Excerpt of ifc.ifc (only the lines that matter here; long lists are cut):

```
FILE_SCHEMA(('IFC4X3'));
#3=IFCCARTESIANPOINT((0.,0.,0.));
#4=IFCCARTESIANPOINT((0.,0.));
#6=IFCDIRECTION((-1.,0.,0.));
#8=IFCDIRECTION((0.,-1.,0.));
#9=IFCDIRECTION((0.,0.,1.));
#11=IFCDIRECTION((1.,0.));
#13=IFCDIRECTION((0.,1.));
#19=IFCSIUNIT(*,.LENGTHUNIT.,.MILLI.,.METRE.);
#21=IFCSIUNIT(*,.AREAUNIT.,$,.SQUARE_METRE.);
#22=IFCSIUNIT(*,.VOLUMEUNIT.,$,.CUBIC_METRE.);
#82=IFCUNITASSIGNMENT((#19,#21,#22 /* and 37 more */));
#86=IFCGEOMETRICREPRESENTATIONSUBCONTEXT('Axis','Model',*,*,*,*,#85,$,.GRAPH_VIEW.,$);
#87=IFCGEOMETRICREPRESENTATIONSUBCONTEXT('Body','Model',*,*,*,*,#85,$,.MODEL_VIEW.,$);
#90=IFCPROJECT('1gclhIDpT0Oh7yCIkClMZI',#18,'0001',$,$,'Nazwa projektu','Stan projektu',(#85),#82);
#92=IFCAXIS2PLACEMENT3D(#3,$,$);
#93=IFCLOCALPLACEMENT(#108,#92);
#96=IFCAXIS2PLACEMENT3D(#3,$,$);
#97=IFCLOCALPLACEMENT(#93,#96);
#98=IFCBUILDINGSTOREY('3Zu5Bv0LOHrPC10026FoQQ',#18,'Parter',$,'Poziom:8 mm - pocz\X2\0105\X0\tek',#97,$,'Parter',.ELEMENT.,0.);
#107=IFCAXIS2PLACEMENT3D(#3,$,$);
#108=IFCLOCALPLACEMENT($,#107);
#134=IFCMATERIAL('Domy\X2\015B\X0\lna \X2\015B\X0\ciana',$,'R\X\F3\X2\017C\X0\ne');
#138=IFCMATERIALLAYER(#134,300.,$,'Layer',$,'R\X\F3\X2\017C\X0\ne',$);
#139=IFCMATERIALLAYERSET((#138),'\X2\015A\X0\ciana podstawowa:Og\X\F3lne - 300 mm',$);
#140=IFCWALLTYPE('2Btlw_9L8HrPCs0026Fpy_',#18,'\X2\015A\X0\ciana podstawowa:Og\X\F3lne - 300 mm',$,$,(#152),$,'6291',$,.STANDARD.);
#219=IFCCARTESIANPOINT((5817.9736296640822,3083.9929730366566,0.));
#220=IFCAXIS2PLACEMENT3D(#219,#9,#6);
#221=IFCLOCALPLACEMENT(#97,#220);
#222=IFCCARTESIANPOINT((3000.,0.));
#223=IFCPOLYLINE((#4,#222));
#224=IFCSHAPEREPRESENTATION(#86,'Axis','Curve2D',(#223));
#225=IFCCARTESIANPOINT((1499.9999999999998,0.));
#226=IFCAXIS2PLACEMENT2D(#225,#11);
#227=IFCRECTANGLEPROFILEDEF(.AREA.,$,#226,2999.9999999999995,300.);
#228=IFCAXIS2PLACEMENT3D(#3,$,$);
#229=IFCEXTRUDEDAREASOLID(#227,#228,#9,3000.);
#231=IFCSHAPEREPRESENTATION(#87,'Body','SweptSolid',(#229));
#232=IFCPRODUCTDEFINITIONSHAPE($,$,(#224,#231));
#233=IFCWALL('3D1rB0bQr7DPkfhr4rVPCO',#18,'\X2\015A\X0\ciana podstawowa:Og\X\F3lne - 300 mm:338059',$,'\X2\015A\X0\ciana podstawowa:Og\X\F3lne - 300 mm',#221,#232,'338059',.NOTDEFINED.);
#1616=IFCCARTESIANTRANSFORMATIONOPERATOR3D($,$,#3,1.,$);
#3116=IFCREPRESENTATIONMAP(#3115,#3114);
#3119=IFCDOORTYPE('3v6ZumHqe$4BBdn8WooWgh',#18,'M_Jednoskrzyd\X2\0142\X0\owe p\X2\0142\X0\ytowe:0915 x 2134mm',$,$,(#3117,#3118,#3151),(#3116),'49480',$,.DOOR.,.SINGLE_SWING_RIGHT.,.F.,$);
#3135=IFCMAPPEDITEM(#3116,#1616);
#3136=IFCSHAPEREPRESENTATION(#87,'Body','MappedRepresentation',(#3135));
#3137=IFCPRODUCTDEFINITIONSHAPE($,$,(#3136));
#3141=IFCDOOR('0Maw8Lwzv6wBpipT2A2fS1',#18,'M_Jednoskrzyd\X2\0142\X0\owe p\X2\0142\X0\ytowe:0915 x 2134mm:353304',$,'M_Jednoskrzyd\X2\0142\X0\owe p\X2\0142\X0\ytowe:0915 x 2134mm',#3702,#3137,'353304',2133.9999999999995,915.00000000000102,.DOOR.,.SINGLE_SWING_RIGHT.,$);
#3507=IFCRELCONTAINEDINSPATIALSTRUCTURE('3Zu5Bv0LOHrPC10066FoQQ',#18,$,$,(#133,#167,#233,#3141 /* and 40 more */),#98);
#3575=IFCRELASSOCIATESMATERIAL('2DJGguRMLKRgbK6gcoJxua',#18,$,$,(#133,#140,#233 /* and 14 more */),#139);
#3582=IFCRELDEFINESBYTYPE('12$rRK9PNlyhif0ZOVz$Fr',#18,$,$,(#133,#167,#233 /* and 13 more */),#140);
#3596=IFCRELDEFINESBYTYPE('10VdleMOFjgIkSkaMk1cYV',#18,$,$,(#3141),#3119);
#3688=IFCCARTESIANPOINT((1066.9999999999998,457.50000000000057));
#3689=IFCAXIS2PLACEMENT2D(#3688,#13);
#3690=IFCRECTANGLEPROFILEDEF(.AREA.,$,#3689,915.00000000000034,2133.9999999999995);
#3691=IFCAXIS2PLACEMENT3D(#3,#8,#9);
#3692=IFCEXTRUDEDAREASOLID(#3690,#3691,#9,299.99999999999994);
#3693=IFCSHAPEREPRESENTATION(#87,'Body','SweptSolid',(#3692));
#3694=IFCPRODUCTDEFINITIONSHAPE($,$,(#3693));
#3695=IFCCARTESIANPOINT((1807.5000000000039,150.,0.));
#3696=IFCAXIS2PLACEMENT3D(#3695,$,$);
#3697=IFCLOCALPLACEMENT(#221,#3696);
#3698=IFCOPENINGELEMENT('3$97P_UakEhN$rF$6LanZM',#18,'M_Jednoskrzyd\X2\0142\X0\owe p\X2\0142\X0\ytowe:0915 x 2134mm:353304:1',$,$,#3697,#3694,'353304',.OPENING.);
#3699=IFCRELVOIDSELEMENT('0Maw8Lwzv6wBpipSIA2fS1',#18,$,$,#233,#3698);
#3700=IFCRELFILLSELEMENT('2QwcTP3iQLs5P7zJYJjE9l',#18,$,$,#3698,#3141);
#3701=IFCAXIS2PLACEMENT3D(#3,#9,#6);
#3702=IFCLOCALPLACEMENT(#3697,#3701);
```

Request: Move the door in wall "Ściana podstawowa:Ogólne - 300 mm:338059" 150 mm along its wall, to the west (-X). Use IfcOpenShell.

```python
import ifcopenshell
import ifcopenshell.api.geometry
import ifcopenshell.util.placement

model = ifcopenshell.open("ifc.ifc")

door = model.by_id(3141)
opening = door.FillsVoids[0].RelatingOpeningElement
wall = opening.VoidsElements[0].RelatingBuildingElement

wall_matrix = ifcopenshell.util.placement.get_local_placement(wall.ObjectPlacement)
shift = wall_matrix[:3, 0] * 150.0
before = ifcopenshell.util.placement.get_local_placement(door.ObjectPlacement)[:3, 3].copy()

# The door is placed relative to its opening, so it follows when the opening moves.
matrix = ifcopenshell.util.placement.get_local_placement(opening.ObjectPlacement)
matrix[:3, 3] += shift
ifcopenshell.api.geometry.edit_object_placement(
    model, product=opening, matrix=matrix, is_si=False, should_transform_children=True
)

after = ifcopenshell.util.placement.get_local_placement(door.ObjectPlacement)[:3, 3]
print("door moved by", (after - before).round(3) + 0.0)

model.write("ifc_edited.ifc")
```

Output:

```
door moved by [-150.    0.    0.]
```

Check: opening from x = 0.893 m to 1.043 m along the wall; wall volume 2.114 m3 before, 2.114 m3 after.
